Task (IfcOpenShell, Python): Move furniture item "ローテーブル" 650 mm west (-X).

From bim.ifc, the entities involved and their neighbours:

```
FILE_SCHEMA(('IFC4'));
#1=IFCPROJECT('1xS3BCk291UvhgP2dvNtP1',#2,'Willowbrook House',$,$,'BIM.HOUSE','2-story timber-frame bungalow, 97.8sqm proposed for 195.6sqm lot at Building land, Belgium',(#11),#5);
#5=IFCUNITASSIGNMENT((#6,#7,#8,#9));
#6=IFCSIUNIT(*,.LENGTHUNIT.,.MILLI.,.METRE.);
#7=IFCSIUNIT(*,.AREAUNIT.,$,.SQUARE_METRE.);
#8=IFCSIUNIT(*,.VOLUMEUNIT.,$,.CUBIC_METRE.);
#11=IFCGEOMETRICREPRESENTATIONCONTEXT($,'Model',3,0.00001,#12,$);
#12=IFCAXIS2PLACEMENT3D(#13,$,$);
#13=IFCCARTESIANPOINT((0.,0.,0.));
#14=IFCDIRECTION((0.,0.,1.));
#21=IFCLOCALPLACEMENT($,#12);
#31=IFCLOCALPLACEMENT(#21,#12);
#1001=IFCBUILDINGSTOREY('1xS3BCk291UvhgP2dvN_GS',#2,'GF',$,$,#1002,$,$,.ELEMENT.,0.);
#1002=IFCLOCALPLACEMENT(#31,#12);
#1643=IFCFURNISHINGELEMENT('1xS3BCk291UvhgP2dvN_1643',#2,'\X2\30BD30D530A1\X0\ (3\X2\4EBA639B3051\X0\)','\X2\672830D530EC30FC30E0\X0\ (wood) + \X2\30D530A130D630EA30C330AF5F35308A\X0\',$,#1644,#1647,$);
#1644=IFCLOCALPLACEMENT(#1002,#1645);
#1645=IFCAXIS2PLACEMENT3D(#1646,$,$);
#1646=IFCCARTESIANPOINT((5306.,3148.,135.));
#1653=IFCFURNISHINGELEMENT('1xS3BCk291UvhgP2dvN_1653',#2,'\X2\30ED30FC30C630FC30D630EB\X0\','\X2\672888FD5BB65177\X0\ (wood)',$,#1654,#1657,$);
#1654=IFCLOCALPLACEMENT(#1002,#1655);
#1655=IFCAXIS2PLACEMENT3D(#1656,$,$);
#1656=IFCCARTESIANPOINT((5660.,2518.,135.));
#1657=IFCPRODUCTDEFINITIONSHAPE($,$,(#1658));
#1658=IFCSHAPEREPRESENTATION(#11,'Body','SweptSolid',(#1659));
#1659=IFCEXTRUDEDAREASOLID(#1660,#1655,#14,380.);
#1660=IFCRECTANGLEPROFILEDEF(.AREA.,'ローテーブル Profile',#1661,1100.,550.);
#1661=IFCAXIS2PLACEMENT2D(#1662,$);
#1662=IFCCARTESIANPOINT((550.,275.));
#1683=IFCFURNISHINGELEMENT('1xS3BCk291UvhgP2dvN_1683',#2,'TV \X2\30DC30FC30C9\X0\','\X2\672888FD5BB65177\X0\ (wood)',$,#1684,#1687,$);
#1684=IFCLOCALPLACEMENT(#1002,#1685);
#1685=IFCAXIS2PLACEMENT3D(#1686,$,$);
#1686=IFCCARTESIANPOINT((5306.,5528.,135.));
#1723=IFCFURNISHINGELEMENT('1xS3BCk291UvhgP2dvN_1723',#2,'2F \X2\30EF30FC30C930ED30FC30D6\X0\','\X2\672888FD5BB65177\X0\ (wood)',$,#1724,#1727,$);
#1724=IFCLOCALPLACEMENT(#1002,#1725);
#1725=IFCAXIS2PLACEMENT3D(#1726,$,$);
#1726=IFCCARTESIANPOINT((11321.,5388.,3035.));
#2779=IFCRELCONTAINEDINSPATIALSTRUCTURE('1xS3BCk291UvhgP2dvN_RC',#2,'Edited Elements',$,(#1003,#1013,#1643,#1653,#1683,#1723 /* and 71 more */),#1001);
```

```python
import ifcopenshell
import ifcopenshell.api.geometry
import ifcopenshell.util.placement
import ifcopenshell.util.unit

model = ifcopenshell.open("bim.ifc")
unit_scale = ifcopenshell.util.unit.calculate_unit_scale(model)

item = model.by_guid("1xS3BCk291UvhgP2dvN_1653")
matrix = ifcopenshell.util.placement.get_local_placement(item.ObjectPlacement)
matrix[0, 3] -= 0.65 / unit_scale
ifcopenshell.api.geometry.edit_object_placement(model, product=item, matrix=matrix, is_si=False)

print(ifcopenshell.util.placement.get_local_placement(item.ObjectPlacement).round(3) + 0.0)

model.write("bim_rev.ifc")
```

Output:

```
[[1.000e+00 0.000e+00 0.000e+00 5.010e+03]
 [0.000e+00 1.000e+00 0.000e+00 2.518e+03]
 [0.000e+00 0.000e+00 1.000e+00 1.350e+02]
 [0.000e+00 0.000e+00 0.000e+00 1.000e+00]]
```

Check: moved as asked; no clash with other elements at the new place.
